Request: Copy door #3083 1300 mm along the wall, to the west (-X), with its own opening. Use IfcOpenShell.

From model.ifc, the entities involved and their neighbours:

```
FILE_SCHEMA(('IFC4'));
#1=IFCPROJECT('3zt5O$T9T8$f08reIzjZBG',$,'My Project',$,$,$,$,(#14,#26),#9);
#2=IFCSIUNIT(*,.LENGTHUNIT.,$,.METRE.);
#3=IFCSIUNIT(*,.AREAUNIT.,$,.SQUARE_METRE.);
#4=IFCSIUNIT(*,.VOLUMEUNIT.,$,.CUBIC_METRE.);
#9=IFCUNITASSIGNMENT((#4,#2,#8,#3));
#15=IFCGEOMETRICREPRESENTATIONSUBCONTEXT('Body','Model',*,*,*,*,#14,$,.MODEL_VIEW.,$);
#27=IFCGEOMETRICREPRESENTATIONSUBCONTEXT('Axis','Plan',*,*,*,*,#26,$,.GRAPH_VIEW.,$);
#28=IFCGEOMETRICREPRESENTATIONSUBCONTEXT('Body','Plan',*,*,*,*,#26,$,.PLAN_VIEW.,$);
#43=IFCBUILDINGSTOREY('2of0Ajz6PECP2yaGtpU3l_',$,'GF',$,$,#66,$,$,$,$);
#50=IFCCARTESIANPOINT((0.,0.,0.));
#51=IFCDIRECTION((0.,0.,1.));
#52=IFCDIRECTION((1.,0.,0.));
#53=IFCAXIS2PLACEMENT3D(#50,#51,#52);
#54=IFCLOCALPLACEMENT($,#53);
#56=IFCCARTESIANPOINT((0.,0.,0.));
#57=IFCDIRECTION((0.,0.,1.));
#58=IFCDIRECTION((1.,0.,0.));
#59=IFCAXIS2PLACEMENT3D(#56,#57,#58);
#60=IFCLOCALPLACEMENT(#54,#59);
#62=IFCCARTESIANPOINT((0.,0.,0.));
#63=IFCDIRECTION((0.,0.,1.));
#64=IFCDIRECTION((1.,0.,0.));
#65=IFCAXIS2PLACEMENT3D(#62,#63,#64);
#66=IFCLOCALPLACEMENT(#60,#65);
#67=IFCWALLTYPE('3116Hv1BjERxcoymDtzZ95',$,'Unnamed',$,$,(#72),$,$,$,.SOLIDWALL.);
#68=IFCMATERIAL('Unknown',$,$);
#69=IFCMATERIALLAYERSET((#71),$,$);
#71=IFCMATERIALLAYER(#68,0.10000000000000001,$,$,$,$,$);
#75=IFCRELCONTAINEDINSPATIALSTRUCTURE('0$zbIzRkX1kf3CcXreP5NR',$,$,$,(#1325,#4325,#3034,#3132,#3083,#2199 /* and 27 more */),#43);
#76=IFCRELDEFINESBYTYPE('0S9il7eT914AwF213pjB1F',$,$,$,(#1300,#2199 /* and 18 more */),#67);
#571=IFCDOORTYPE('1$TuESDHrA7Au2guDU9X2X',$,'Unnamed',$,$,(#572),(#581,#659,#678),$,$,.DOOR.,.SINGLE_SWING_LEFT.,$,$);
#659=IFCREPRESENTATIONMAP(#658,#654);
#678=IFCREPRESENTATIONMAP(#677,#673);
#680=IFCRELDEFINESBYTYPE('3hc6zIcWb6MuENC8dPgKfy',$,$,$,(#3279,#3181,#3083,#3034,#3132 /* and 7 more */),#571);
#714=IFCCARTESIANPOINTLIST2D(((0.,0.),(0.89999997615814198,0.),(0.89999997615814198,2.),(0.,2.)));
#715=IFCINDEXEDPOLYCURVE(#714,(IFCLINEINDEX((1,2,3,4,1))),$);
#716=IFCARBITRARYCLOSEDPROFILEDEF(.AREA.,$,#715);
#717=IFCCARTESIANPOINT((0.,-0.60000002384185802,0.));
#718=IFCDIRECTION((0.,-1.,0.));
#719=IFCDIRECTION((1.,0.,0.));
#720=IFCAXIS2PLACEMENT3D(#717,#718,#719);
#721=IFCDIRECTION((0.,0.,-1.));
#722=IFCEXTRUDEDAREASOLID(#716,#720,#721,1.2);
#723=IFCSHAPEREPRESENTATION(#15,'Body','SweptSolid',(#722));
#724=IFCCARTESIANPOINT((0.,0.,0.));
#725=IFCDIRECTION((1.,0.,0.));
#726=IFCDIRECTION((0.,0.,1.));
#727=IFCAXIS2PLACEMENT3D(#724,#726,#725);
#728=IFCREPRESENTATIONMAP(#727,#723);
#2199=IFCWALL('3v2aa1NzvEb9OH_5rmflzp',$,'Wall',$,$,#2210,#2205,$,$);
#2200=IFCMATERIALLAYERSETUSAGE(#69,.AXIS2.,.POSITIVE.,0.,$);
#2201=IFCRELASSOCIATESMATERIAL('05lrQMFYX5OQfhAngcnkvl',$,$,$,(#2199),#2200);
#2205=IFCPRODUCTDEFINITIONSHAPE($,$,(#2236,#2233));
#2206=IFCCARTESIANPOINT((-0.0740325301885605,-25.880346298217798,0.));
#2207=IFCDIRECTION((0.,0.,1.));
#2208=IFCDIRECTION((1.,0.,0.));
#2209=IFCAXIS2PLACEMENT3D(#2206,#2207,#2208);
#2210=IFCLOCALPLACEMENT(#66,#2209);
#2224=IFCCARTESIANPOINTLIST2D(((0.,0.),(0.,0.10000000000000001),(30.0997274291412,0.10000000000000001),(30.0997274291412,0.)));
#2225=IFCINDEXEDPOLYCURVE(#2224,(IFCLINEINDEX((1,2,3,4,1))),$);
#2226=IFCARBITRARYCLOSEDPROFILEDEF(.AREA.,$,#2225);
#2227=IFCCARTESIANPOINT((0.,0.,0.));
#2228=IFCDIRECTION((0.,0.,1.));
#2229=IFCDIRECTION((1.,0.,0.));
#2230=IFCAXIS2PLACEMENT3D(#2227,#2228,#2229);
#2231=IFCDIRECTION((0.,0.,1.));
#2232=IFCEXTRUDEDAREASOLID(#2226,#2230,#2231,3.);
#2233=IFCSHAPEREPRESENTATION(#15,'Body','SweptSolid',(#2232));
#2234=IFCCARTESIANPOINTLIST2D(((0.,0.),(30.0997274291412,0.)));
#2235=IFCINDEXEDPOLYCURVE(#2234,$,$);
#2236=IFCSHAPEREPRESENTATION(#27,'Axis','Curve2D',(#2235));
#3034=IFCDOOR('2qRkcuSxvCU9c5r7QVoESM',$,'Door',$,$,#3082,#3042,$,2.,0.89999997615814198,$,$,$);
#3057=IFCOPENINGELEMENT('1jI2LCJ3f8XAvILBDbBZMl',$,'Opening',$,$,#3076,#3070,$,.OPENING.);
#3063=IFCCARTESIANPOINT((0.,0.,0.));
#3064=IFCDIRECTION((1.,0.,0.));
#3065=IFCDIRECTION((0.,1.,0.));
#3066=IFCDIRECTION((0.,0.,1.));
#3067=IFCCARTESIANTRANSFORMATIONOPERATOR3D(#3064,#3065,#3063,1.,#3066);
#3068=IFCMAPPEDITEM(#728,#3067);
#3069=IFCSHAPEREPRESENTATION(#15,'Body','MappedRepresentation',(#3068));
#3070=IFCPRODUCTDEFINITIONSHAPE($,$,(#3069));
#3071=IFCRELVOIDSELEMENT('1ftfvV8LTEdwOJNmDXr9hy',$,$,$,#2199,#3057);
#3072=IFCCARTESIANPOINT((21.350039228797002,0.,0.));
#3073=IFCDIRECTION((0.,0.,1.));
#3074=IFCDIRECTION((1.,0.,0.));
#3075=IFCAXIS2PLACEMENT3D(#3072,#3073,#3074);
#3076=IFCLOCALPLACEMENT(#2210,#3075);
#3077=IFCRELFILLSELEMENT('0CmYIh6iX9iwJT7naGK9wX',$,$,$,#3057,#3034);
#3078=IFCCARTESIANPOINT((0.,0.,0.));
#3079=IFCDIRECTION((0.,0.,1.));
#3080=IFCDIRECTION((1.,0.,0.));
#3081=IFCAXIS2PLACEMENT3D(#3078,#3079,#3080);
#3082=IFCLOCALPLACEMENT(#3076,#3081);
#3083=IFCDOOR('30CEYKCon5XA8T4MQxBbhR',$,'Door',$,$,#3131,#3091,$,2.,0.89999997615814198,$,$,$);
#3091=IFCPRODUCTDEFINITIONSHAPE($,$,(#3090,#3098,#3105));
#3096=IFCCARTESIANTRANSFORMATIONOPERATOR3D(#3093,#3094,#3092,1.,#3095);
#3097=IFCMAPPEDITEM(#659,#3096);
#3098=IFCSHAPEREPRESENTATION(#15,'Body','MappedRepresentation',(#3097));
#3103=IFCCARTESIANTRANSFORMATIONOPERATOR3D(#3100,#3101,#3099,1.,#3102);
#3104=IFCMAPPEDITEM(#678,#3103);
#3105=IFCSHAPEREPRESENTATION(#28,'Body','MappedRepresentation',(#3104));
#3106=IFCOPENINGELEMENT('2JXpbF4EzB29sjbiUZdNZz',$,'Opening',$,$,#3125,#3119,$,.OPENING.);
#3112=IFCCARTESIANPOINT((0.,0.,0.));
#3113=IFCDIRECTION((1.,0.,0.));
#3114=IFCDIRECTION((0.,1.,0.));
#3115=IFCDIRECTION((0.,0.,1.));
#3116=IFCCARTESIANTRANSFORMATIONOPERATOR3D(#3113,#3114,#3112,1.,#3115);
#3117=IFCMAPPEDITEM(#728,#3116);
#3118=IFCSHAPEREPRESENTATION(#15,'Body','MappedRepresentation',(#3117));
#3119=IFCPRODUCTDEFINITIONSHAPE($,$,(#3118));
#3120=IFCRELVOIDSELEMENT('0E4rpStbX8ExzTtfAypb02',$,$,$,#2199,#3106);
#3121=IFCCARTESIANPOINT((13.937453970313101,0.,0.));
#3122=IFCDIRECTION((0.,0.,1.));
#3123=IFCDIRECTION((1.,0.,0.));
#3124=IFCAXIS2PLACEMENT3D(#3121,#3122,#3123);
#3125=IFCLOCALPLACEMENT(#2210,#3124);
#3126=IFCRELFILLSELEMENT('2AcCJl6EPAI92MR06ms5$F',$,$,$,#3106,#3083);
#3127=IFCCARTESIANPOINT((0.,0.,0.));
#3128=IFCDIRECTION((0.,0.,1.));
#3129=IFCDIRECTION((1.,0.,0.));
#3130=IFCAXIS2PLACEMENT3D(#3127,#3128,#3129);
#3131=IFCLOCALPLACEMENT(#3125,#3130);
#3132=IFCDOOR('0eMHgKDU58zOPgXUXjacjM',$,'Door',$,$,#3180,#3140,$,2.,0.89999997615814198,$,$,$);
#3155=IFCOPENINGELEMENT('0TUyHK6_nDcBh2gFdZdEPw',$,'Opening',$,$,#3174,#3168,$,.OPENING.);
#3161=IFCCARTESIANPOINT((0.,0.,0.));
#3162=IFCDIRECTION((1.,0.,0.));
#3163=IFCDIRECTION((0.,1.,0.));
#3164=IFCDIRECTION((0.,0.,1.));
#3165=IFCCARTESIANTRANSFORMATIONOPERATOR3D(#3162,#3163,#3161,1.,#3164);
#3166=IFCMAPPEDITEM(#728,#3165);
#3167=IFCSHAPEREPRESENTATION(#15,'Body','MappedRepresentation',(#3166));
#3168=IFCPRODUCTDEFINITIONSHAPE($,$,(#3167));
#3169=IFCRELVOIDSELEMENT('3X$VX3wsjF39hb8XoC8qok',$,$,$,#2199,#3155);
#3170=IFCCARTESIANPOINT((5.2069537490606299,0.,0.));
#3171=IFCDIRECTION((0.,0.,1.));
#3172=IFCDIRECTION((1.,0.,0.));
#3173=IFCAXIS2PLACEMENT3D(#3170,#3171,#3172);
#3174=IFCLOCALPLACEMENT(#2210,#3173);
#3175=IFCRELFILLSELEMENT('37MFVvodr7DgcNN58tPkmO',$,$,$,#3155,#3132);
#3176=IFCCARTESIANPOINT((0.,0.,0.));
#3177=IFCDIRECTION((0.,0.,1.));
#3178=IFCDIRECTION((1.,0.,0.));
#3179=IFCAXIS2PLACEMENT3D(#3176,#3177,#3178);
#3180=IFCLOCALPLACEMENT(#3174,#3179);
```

```python
import ifcopenshell
import ifcopenshell.api.feature
import ifcopenshell.api.geometry
import ifcopenshell.api.root
import ifcopenshell.geom
import ifcopenshell.util.element
import ifcopenshell.util.placement
import ifcopenshell.util.shape
import ifcopenshell.util.unit

model = ifcopenshell.open("model.ifc")
unit_scale = ifcopenshell.util.unit.calculate_unit_scale(model)
settings = ifcopenshell.geom.settings()


def volume(element):
    """Net volume in cubic metres, openings subtracted."""
    shape = ifcopenshell.geom.create_shape(settings, element)
    return ifcopenshell.util.shape.get_volume(shape.geometry)


door = model.by_guid("30CEYKCon5XA8T4MQxBbhR")
opening = door.FillsVoids[0].RelatingOpeningElement
wall = opening.VoidsElements[0].RelatingBuildingElement
before = volume(wall)
shift = ifcopenshell.util.placement.get_local_placement(wall.ObjectPlacement)[:3, 0] * -1.3 / unit_scale

# copy_class copies the void relationship, type, container and properties, but no geometry.
new_opening = ifcopenshell.api.root.copy_class(model, product=opening)
new_opening.Representation = ifcopenshell.util.element.copy_deep(
    model, opening.Representation, exclude=["IfcGeometricRepresentationContext", "IfcRepresentationMap"]
)
new_door = ifcopenshell.api.root.copy_class(model, product=door)
new_door.Representation = ifcopenshell.util.element.copy_deep(
    model, door.Representation, exclude=["IfcGeometricRepresentationContext", "IfcRepresentationMap"]
)
ifcopenshell.api.feature.add_filling(model, opening=new_opening, element=new_door)

for old, new in ((opening, new_opening), (door, new_door)):
    matrix = ifcopenshell.util.placement.get_local_placement(old.ObjectPlacement)
    matrix[:3, 3] += shift
    ifcopenshell.api.geometry.edit_object_placement(model, product=new, matrix=matrix, is_si=False)

after = volume(wall)

print(f"wall volume {before:.3f} -> {after:.3f} m3")

model.write("model-out.ifc")
```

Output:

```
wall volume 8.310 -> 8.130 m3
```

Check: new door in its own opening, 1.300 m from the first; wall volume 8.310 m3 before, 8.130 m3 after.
